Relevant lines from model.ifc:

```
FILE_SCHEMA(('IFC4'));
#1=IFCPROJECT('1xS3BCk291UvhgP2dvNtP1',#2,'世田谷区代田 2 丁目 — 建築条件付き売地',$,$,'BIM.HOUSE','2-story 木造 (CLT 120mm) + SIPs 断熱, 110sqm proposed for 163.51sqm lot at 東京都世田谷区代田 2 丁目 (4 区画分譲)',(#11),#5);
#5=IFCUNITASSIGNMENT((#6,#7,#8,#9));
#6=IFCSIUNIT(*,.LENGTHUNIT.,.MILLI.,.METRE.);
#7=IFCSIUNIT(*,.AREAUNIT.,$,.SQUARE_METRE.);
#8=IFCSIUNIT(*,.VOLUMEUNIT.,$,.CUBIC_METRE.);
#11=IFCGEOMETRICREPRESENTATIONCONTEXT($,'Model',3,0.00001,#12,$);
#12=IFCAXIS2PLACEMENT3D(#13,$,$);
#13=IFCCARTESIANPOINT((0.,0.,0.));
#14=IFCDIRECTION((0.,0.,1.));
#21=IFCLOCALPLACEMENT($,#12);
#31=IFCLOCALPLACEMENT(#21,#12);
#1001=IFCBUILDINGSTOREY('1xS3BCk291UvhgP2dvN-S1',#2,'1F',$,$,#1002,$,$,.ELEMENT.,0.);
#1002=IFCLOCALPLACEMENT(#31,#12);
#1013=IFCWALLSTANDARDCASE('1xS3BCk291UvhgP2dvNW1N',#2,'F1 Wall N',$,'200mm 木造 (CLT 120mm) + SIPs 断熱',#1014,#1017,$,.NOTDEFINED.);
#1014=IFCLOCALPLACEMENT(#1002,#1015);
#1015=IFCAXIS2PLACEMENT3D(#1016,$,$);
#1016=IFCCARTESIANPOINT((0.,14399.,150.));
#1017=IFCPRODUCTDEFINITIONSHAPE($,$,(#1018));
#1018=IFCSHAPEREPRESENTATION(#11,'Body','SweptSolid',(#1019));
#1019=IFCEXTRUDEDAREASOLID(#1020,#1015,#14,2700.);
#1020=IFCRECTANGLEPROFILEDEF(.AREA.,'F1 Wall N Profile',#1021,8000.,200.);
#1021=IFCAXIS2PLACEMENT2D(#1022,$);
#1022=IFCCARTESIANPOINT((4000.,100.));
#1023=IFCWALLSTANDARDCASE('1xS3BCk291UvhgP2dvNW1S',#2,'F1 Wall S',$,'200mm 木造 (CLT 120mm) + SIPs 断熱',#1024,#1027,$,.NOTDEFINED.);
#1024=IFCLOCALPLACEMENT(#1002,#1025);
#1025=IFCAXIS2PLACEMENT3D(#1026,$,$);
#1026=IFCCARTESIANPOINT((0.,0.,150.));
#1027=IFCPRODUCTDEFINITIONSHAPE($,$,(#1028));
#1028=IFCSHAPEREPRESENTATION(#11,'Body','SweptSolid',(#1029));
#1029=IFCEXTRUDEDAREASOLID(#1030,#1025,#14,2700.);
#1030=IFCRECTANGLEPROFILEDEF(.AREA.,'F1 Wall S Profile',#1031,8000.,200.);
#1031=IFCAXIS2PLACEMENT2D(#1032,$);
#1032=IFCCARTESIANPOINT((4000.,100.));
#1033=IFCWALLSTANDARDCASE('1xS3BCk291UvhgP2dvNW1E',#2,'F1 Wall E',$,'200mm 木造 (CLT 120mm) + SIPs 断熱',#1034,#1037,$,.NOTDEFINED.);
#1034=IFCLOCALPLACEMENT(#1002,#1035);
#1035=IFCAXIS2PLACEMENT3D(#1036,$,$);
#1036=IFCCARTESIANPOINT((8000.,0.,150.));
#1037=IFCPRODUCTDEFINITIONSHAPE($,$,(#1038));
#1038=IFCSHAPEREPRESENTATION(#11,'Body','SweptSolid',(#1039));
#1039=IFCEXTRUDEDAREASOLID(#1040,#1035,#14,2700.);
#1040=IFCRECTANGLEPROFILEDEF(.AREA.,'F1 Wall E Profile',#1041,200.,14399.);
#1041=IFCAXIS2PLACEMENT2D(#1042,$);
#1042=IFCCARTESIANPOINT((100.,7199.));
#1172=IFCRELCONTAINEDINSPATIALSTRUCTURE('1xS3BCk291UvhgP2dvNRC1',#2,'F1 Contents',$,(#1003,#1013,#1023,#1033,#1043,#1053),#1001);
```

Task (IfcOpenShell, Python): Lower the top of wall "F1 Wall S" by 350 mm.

```python
import ifcopenshell
import ifcopenshell.geom
import ifcopenshell.util.shape
import ifcopenshell.util.unit

model = ifcopenshell.open("model.ifc")
unit_scale = ifcopenshell.util.unit.calculate_unit_scale(model)
settings = ifcopenshell.geom.settings()


def volume(element):
    """Net volume in cubic metres, openings subtracted."""
    shape = ifcopenshell.geom.create_shape(settings, element)
    return ifcopenshell.util.shape.get_volume(shape.geometry)


wall = model.by_guid("1xS3BCk291UvhgP2dvNW1S")
before = volume(wall)

body = next(r for r in wall.Representation.Representations if r.RepresentationIdentifier == "Body")
solid = body.Items[0]
old_height = solid.Depth
solid.Depth -= 0.35 / unit_scale
after = volume(wall)

print(f"height {old_height:g} -> {solid.Depth:g}, volume {before:.3f} -> {after:.3f} m3")

model.write("model_v2.ifc")
```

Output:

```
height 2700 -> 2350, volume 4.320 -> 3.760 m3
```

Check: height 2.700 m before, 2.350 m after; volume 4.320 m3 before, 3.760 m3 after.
